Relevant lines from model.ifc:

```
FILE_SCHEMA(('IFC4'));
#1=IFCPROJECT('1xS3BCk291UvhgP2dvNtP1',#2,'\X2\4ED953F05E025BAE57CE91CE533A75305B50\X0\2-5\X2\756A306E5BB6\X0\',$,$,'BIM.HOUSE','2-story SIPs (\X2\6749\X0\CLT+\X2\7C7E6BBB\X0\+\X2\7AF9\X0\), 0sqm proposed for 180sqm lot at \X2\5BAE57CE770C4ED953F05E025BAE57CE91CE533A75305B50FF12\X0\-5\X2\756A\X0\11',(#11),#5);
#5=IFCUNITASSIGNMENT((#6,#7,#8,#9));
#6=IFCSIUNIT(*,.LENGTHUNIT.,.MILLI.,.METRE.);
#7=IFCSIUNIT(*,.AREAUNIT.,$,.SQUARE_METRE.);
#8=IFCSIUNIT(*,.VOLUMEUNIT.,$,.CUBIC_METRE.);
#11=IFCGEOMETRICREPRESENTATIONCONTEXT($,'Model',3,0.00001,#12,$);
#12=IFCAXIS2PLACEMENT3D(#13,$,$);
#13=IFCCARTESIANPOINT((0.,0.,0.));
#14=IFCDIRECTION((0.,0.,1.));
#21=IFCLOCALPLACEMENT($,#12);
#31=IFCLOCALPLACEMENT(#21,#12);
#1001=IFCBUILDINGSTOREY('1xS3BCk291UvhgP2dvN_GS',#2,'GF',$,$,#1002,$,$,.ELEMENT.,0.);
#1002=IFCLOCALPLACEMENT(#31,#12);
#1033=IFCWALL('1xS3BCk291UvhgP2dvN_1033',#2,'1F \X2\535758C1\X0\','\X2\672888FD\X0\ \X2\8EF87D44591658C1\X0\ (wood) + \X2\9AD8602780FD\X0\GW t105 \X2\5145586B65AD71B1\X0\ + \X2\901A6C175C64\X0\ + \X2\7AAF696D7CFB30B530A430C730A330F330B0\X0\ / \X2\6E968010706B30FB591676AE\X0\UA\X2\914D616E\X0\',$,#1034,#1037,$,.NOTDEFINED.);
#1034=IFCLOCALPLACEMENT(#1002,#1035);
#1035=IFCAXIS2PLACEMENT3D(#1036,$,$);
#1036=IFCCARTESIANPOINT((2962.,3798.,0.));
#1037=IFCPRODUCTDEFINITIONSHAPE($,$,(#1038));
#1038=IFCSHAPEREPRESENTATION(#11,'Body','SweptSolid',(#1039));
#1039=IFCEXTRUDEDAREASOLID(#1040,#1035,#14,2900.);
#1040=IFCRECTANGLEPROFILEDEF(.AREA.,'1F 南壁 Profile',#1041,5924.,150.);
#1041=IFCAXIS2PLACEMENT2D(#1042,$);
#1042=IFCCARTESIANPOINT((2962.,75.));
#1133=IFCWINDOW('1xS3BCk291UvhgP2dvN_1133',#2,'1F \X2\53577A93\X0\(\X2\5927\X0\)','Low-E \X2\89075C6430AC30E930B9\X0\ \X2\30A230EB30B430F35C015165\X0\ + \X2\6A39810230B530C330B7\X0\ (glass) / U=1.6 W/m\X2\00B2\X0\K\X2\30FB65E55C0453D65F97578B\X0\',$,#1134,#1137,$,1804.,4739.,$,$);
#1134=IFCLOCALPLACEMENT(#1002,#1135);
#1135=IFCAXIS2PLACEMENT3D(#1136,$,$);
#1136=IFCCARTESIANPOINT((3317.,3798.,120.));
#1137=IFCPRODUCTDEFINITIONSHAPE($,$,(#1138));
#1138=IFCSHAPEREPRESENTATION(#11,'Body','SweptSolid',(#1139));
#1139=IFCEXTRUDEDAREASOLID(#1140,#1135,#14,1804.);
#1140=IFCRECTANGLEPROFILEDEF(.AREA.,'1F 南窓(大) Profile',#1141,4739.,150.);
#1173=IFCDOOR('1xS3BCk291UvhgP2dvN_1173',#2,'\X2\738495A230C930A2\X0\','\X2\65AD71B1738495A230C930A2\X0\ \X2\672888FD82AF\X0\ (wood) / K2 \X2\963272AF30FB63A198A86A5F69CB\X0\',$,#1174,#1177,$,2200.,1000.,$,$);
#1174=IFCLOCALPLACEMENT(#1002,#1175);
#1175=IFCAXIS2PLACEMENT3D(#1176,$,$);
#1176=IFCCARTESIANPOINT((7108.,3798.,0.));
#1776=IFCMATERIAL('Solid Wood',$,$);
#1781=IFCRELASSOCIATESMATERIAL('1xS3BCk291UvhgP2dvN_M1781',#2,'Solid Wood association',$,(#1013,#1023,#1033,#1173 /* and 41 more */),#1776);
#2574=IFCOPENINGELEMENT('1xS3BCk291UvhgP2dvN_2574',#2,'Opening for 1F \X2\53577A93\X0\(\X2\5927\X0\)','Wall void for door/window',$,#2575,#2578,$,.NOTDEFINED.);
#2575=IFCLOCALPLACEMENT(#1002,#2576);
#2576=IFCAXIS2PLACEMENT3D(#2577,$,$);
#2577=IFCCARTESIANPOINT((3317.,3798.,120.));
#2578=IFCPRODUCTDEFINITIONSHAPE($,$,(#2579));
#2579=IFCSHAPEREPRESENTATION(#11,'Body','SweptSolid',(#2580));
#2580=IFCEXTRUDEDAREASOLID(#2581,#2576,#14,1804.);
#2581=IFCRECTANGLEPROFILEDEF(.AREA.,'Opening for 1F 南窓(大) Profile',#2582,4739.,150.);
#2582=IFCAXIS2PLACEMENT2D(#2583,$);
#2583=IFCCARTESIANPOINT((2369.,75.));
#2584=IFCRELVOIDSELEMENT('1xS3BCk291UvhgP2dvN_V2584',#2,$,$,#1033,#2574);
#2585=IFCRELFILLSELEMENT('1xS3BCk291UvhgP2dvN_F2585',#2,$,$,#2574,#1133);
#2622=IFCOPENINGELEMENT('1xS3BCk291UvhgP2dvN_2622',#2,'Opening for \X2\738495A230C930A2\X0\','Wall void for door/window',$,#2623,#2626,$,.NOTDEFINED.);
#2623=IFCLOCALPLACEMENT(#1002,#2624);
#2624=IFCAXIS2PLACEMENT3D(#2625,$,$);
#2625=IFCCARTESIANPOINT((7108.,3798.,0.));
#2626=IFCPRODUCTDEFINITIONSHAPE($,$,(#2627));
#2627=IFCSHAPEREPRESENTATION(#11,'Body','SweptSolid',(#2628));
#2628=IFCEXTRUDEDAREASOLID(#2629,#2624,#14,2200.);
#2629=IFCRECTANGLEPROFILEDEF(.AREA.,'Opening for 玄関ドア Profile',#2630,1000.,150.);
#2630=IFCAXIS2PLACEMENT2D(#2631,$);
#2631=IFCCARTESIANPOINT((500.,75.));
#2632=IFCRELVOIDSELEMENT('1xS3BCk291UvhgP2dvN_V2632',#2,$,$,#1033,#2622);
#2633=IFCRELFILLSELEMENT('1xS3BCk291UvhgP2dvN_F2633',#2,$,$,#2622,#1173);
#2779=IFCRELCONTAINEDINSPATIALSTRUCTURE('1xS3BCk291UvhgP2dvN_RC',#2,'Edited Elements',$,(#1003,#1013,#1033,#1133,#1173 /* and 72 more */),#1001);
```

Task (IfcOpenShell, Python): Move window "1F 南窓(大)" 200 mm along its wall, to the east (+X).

```python
import ifcopenshell
import ifcopenshell.api.geometry
import ifcopenshell.util.placement

model = ifcopenshell.open("model.ifc")

window = model.by_guid("1xS3BCk291UvhgP2dvN_1133")
opening = window.FillsVoids[0].RelatingOpeningElement
wall = opening.VoidsElements[0].RelatingBuildingElement

wall_matrix = ifcopenshell.util.placement.get_local_placement(wall.ObjectPlacement)
shift = wall_matrix[:3, 0] * 200.0
before = ifcopenshell.util.placement.get_local_placement(window.ObjectPlacement)[:3, 3].copy()

# The window is not placed relative to its opening, so move both.
for product in (opening, window):
    matrix = ifcopenshell.util.placement.get_local_placement(product.ObjectPlacement)
    matrix[:3, 3] += shift
    ifcopenshell.api.geometry.edit_object_placement(model, product=product, matrix=matrix, is_si=False)

after = ifcopenshell.util.placement.get_local_placement(window.ObjectPlacement)[:3, 3]
print("window moved by", (after - before).round(3) + 0.0)

model.write("model_edited.ifc")
```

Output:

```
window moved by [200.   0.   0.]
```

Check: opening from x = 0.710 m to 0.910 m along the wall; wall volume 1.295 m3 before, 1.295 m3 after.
